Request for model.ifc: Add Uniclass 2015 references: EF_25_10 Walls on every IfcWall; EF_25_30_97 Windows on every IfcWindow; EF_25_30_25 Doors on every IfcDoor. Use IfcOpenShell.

First a look at what the model holds.

```python
import ifcopenshell

model = ifcopenshell.open("model.ifc")
print(model.schema)
print("classifications:", [c.Name for c in model.by_type("IfcClassification")])
for ifc_class in ("IfcDoor", "IfcRoof", "IfcStair", "IfcWall", "IfcWindow"):
    print(ifc_class, len(model.by_type(ifc_class)))
```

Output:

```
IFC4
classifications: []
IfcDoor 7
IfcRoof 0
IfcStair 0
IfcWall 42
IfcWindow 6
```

```python
import ifcopenshell
import ifcopenshell.api.classification

model = ifcopenshell.open("model.ifc")

system = ifcopenshell.api.classification.add_classification(model, classification="Uniclass 2015")

codes = {
    "IfcWall": ("EF_25_10", "Walls"),
    "IfcWindow": ("EF_25_30_97", "Windows"),
    "IfcDoor": ("EF_25_30_25", "Doors"),
}
for ifc_class, (code, name) in codes.items():
    products = model.by_type(ifc_class)
    ifcopenshell.api.classification.add_reference(
        model, products=products, classification=system, identification=code, name=name
    )
    print(code, len(products))

model.write("model_rev.ifc")
```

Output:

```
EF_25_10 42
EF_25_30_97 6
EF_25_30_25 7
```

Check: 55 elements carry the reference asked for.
